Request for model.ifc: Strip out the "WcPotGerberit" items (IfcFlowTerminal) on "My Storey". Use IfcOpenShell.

First a look at what the model holds.

```python
import ifcopenshell
import ifcopenshell.util.element

model = ifcopenshell.open("model.ifc")
print(model.schema)
storey = next(s for s in model.by_type("IfcBuildingStorey") if s.Name == "My Storey")
terminals = [e for e in ifcopenshell.util.element.get_decomposition(storey) if e.is_a("IfcFlowTerminal")]
seen = {}
for e in terminals:
    element_type = ifcopenshell.util.element.get_type(e)
    name = element_type.Name if element_type not in (None, e) else None
    seen[name] = seen.get(name, 0) + 1
for name, count in sorted(seen.items(), key=str):
    print(count, "x", name)
```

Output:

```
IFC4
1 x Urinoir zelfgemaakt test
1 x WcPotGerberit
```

```python
import ifcopenshell
import ifcopenshell.api.root
import ifcopenshell.util.element

model = ifcopenshell.open("model.ifc")

storey = next(s for s in model.by_type("IfcBuildingStorey") if s.Name == "My Storey")
terminals = [e for e in ifcopenshell.util.element.get_decomposition(storey) if e.is_a("IfcFlowTerminal")]
targets = [e for e in terminals if (t := ifcopenshell.util.element.get_type(e)) not in (None, e) and t.Name == "WcPotGerberit"]

for e in targets:
    ifcopenshell.api.root.remove_product(model, product=e)
print(len(targets), "removed")

model.write("model_v2.ifc")
```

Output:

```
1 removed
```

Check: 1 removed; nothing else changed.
